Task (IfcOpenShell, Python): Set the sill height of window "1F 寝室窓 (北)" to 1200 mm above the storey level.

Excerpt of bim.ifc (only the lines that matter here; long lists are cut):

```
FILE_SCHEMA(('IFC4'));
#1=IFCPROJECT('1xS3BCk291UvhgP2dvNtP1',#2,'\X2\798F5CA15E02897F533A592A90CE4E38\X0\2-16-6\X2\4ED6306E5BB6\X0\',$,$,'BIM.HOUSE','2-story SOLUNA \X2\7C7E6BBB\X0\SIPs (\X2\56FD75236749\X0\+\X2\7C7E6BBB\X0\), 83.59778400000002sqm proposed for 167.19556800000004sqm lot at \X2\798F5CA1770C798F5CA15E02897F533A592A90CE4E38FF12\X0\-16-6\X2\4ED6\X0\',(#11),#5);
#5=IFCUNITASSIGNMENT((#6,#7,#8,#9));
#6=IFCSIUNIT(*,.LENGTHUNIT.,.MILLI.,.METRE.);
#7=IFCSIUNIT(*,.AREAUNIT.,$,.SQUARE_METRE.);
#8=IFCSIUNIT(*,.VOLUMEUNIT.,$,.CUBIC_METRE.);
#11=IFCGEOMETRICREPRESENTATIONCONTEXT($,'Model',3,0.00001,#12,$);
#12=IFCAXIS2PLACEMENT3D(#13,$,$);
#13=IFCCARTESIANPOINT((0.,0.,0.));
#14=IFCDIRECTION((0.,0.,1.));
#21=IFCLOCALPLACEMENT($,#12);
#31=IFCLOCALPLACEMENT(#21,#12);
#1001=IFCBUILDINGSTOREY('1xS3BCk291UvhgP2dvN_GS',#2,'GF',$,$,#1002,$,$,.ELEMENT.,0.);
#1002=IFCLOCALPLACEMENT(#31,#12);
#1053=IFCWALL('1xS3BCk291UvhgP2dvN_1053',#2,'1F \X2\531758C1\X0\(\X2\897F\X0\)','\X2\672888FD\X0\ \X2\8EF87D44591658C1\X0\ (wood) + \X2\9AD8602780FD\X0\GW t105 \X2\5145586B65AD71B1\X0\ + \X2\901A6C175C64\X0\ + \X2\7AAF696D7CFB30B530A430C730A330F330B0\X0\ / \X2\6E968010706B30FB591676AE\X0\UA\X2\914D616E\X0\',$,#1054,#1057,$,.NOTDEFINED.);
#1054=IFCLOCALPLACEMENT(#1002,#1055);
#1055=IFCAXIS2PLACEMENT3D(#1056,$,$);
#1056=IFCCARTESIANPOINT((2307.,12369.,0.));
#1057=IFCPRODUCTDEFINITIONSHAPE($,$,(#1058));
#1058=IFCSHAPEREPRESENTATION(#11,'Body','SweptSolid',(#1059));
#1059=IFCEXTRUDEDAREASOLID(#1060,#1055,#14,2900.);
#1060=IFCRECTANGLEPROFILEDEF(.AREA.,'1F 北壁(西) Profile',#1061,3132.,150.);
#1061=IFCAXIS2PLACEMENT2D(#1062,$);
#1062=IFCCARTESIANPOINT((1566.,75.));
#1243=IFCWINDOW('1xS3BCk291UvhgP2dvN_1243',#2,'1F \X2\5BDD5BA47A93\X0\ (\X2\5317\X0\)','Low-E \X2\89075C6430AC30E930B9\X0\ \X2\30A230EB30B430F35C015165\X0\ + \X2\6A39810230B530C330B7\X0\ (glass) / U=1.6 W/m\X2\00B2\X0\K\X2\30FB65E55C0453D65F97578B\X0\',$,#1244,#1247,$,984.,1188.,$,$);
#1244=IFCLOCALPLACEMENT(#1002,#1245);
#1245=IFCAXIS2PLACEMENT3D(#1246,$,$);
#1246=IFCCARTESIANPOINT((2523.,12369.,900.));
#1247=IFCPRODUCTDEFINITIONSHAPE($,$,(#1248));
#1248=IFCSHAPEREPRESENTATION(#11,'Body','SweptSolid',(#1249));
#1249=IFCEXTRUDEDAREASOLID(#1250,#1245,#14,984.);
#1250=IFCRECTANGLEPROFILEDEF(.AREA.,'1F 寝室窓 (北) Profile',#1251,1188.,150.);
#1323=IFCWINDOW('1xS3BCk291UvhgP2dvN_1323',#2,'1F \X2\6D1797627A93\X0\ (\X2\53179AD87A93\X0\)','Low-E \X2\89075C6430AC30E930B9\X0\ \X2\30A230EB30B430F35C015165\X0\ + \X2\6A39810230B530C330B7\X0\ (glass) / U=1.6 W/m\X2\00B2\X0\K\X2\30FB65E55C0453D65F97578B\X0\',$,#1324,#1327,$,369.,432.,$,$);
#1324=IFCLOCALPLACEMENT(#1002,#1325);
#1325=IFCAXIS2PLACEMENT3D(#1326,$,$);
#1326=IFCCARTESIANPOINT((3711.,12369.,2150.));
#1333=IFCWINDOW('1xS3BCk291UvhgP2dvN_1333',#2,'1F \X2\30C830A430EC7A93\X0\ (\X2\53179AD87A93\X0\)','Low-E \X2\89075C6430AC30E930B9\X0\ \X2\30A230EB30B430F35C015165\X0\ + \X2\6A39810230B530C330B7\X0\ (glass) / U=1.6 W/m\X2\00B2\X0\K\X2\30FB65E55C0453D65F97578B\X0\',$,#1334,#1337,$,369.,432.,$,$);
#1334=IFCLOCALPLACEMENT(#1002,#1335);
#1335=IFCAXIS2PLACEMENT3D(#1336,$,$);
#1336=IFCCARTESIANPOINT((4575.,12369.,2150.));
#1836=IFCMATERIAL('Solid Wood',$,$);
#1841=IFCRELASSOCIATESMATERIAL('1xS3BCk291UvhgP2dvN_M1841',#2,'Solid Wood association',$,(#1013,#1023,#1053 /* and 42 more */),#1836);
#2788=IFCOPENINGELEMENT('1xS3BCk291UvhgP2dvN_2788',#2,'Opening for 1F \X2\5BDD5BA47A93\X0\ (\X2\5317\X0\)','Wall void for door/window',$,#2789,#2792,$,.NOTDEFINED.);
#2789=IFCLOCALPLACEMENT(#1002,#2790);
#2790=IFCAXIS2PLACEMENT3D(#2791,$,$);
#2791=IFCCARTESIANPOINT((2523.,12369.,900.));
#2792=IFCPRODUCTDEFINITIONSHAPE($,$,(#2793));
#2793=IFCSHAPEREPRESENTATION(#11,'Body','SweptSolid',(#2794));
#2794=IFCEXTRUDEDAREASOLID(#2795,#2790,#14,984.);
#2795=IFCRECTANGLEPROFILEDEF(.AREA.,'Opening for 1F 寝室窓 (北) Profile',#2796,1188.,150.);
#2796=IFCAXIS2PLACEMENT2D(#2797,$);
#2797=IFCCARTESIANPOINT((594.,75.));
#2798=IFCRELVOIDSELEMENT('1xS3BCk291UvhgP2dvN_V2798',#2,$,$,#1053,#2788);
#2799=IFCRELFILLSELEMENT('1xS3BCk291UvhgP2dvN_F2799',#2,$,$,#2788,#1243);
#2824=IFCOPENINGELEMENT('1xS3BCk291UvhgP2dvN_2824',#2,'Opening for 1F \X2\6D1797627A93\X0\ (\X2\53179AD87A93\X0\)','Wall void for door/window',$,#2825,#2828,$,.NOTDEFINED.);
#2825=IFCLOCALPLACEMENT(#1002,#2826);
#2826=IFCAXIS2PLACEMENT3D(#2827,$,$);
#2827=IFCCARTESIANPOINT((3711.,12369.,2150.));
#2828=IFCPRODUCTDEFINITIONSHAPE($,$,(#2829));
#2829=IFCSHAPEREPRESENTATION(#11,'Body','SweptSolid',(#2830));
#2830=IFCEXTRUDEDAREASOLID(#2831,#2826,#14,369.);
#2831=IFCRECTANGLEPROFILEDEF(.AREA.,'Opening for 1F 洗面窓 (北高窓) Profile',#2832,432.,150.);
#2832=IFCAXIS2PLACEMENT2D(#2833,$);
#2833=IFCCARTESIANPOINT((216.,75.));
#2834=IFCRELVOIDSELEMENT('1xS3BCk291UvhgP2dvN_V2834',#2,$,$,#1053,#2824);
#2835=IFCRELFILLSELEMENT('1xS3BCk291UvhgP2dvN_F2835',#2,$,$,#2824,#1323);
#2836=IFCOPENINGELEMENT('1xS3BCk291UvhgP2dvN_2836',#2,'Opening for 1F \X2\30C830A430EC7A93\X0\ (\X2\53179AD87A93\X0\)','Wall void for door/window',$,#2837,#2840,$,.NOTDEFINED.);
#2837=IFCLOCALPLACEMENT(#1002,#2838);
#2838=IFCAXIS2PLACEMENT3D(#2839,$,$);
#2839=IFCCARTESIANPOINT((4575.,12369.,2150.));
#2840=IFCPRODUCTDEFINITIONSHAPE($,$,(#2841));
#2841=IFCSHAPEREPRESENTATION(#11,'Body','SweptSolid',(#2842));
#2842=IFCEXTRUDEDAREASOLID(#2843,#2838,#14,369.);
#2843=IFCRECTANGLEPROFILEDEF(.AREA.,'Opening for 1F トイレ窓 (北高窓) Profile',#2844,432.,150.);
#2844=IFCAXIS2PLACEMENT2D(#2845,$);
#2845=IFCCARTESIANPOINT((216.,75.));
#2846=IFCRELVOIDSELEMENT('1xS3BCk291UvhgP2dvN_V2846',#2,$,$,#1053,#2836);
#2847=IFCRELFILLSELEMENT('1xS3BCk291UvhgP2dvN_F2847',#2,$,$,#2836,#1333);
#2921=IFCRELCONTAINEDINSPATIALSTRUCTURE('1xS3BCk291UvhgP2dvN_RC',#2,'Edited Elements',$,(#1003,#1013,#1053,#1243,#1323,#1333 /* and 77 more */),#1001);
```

```python
import numpy as np
import ifcopenshell
import ifcopenshell.api.geometry
import ifcopenshell.geom
import ifcopenshell.util.element
import ifcopenshell.util.placement
import ifcopenshell.util.shape
import ifcopenshell.util.unit

model = ifcopenshell.open("bim.ifc")
unit_scale = ifcopenshell.util.unit.calculate_unit_scale(model)

window = model.by_id(1243)
opening = window.FillsVoids[0].RelatingOpeningElement
storey = ifcopenshell.util.element.get_container(window, ifc_class="IfcBuildingStorey")
level = ifcopenshell.util.placement.get_local_placement(storey.ObjectPlacement)[2, 3]

# The opening's origin need not be at the sill, so measure its lowest point.
shape = ifcopenshell.geom.create_shape(ifcopenshell.geom.settings(), opening)
bottom = ifcopenshell.util.shape.get_shape_bottom_elevation(shape, shape.geometry) / unit_scale
dz = level + 1.2 / unit_scale - bottom

shift = np.array([0.0, 0.0, dz])
# The window is not placed relative to its opening, so move both.
for product in (opening, window):
    matrix = ifcopenshell.util.placement.get_local_placement(product.ObjectPlacement)
    matrix[:3, 3] += shift
    ifcopenshell.api.geometry.edit_object_placement(model, product=product, matrix=matrix, is_si=False)

print(f"moved by {dz * unit_scale:+.3f} m")

model.write("bim-out.ifc")
```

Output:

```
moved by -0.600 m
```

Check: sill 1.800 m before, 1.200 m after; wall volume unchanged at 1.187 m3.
